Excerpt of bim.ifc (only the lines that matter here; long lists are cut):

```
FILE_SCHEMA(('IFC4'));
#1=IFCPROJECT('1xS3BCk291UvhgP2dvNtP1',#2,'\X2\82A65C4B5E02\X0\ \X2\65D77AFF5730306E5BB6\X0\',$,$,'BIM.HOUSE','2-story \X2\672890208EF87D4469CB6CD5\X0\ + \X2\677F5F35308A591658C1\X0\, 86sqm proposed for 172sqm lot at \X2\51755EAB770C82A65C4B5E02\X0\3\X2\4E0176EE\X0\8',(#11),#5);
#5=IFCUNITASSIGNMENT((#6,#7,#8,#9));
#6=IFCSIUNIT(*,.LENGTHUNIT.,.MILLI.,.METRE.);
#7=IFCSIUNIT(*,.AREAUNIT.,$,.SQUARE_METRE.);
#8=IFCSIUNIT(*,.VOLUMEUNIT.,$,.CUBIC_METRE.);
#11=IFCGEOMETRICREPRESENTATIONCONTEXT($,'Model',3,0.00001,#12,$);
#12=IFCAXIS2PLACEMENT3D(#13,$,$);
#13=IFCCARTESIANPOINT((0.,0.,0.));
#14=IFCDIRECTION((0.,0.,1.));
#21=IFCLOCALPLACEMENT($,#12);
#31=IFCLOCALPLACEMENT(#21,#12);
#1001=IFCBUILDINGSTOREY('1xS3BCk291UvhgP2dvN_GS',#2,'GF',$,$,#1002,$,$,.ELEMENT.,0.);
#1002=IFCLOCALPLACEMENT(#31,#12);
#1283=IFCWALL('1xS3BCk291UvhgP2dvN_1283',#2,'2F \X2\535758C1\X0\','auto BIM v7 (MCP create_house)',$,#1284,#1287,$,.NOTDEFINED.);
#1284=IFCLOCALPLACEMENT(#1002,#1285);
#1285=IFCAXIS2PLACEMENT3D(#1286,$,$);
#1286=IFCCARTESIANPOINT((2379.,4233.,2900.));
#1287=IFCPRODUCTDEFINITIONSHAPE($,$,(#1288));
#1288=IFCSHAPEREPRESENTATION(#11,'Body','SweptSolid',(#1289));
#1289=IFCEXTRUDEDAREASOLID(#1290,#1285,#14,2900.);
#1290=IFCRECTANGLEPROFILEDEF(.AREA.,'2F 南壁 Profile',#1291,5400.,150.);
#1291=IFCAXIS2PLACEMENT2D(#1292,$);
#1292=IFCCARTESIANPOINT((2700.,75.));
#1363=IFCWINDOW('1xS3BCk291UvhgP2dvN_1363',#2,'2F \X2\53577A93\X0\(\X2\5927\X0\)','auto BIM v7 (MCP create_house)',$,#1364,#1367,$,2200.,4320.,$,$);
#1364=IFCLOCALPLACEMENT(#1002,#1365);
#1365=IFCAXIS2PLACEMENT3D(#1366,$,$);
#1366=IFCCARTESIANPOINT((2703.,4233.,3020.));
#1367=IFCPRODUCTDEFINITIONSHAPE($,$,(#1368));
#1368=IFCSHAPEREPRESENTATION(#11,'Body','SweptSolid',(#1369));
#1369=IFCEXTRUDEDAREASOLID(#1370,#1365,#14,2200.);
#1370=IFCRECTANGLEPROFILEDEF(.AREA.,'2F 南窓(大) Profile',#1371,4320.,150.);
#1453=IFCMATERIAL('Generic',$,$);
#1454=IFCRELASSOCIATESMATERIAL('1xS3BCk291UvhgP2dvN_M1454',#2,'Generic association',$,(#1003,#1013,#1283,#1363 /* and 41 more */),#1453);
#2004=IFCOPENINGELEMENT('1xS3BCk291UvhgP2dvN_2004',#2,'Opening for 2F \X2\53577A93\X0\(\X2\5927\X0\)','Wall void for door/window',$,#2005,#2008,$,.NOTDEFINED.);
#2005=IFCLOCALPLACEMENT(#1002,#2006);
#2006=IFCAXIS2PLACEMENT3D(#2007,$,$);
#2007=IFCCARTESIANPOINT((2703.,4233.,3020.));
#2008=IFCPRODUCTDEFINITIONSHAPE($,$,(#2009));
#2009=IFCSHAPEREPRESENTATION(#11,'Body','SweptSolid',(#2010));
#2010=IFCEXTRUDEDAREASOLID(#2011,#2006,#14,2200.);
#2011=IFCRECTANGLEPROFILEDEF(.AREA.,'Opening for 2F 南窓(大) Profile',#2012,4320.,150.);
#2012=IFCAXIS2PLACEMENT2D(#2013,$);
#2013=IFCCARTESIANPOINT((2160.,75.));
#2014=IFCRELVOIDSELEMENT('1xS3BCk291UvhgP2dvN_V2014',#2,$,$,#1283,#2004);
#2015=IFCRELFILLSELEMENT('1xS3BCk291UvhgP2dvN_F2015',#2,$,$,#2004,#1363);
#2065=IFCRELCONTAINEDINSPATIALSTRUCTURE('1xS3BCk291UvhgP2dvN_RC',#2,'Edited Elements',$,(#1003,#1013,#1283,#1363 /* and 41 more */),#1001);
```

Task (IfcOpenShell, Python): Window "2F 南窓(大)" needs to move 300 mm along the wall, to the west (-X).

```python
import ifcopenshell
import ifcopenshell.api.geometry
import ifcopenshell.util.placement
import ifcopenshell.util.unit

model = ifcopenshell.open("bim.ifc")
unit_scale = ifcopenshell.util.unit.calculate_unit_scale(model)

window = model.by_id(1363)
opening = window.FillsVoids[0].RelatingOpeningElement
wall = opening.VoidsElements[0].RelatingBuildingElement

wall_matrix = ifcopenshell.util.placement.get_local_placement(wall.ObjectPlacement)
shift = wall_matrix[:3, 0] * -0.3 / unit_scale
before = ifcopenshell.util.placement.get_local_placement(window.ObjectPlacement)[:3, 3].copy()

# The window is not placed relative to its opening, so move both.
for product in (opening, window):
    matrix = ifcopenshell.util.placement.get_local_placement(product.ObjectPlacement)
    matrix[:3, 3] += shift
    ifcopenshell.api.geometry.edit_object_placement(model, product=product, matrix=matrix, is_si=False)

after = ifcopenshell.util.placement.get_local_placement(window.ObjectPlacement)[:3, 3]
print("window moved by", (after - before).round(3) + 0.0)

model.write("bim-out.ifc")
```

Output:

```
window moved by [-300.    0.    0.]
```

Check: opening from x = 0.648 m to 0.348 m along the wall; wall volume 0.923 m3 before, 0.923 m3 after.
